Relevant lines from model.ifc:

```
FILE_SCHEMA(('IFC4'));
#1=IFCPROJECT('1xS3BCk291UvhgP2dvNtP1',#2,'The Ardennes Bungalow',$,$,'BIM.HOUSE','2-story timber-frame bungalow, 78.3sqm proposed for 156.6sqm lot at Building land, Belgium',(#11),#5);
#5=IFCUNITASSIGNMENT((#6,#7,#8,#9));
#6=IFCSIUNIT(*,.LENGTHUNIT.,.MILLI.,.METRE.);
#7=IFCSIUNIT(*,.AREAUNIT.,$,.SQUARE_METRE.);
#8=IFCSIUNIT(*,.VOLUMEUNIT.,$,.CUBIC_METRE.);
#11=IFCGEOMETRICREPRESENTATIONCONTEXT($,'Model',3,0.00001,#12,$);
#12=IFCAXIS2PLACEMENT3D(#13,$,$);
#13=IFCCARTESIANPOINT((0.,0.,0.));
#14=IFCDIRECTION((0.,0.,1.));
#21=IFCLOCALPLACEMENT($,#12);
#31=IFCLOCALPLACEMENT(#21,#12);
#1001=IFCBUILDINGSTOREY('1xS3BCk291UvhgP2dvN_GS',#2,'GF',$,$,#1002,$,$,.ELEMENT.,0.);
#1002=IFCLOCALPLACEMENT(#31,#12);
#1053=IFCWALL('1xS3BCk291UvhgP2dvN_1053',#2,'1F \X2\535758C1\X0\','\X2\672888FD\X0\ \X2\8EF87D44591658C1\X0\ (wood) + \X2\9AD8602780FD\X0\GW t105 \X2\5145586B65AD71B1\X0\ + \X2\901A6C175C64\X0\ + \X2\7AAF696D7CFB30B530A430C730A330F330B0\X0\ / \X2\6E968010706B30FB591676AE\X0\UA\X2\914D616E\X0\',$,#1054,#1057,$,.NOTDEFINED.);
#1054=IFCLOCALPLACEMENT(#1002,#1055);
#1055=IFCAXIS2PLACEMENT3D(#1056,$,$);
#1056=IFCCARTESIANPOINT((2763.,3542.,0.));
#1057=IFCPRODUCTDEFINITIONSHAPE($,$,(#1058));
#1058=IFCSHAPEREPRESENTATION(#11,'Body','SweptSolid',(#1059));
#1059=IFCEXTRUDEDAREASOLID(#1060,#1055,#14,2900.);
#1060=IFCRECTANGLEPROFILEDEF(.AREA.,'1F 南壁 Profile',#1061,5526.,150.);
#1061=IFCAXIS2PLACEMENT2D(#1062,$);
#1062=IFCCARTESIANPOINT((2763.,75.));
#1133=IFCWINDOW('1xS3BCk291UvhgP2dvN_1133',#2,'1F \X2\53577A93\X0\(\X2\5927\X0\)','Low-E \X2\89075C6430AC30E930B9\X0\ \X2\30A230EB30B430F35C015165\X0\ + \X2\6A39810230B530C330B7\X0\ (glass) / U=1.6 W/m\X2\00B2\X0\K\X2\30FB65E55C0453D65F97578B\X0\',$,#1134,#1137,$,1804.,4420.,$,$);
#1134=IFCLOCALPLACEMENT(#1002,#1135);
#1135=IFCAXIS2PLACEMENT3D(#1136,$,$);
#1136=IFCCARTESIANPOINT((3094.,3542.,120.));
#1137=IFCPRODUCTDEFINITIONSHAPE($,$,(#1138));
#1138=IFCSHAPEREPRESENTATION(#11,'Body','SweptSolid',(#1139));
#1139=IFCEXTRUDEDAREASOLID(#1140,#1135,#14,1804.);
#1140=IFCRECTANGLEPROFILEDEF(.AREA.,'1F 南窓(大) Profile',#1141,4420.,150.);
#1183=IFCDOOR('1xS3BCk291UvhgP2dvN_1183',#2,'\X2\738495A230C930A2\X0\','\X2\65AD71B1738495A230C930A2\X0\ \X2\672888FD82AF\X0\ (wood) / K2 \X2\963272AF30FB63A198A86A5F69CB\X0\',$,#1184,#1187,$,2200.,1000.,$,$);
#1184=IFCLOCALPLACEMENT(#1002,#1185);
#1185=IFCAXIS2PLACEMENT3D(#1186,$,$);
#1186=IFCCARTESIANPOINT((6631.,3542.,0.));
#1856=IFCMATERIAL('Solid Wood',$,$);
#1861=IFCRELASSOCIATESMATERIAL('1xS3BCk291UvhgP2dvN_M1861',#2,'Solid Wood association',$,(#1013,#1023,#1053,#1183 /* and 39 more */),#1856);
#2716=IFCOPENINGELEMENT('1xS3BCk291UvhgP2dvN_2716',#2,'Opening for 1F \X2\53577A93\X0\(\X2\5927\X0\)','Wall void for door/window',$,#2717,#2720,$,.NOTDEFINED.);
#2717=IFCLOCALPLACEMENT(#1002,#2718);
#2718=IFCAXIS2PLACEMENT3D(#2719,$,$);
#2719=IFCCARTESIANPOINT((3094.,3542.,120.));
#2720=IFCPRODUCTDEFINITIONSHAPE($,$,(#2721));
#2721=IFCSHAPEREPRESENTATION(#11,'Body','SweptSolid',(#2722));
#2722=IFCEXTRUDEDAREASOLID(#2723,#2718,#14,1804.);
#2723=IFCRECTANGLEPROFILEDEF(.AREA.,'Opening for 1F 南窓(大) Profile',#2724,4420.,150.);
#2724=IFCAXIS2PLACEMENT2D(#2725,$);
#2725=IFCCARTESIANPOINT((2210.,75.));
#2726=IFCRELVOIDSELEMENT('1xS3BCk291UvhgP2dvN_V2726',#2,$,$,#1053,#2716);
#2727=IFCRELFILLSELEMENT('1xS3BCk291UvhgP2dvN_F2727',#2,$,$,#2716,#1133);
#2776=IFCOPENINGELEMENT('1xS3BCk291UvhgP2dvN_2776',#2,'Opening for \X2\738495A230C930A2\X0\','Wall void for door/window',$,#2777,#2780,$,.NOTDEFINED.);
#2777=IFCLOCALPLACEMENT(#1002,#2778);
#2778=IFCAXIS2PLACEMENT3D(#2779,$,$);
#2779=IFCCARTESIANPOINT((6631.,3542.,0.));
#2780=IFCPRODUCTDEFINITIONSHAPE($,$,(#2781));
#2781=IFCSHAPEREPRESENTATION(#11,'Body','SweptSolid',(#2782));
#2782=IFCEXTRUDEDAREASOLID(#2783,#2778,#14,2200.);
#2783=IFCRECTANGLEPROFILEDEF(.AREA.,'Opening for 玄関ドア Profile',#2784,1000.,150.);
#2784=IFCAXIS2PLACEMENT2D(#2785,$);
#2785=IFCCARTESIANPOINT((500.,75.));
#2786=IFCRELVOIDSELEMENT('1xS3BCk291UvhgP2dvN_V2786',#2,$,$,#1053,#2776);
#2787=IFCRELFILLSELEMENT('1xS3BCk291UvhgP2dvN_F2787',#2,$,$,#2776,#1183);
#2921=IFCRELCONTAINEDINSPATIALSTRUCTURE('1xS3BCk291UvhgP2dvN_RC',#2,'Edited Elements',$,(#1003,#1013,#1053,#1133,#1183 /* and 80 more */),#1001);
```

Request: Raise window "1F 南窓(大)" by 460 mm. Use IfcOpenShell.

```python
import numpy as np
import ifcopenshell
import ifcopenshell.api.geometry
import ifcopenshell.util.placement
import ifcopenshell.util.unit

model = ifcopenshell.open("model.ifc")
unit_scale = ifcopenshell.util.unit.calculate_unit_scale(model)

window = model.by_guid("1xS3BCk291UvhgP2dvN_1133")
opening = window.FillsVoids[0].RelatingOpeningElement
dz = 460.0

shift = np.array([0.0, 0.0, dz])
# The window is not placed relative to its opening, so move both.
for product in (opening, window):
    matrix = ifcopenshell.util.placement.get_local_placement(product.ObjectPlacement)
    matrix[:3, 3] += shift
    ifcopenshell.api.geometry.edit_object_placement(model, product=product, matrix=matrix, is_si=False)

print(f"moved by {dz * unit_scale:+.3f} m")

model.write("model_rev.ifc")
```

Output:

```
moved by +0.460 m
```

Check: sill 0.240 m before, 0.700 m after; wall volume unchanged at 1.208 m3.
